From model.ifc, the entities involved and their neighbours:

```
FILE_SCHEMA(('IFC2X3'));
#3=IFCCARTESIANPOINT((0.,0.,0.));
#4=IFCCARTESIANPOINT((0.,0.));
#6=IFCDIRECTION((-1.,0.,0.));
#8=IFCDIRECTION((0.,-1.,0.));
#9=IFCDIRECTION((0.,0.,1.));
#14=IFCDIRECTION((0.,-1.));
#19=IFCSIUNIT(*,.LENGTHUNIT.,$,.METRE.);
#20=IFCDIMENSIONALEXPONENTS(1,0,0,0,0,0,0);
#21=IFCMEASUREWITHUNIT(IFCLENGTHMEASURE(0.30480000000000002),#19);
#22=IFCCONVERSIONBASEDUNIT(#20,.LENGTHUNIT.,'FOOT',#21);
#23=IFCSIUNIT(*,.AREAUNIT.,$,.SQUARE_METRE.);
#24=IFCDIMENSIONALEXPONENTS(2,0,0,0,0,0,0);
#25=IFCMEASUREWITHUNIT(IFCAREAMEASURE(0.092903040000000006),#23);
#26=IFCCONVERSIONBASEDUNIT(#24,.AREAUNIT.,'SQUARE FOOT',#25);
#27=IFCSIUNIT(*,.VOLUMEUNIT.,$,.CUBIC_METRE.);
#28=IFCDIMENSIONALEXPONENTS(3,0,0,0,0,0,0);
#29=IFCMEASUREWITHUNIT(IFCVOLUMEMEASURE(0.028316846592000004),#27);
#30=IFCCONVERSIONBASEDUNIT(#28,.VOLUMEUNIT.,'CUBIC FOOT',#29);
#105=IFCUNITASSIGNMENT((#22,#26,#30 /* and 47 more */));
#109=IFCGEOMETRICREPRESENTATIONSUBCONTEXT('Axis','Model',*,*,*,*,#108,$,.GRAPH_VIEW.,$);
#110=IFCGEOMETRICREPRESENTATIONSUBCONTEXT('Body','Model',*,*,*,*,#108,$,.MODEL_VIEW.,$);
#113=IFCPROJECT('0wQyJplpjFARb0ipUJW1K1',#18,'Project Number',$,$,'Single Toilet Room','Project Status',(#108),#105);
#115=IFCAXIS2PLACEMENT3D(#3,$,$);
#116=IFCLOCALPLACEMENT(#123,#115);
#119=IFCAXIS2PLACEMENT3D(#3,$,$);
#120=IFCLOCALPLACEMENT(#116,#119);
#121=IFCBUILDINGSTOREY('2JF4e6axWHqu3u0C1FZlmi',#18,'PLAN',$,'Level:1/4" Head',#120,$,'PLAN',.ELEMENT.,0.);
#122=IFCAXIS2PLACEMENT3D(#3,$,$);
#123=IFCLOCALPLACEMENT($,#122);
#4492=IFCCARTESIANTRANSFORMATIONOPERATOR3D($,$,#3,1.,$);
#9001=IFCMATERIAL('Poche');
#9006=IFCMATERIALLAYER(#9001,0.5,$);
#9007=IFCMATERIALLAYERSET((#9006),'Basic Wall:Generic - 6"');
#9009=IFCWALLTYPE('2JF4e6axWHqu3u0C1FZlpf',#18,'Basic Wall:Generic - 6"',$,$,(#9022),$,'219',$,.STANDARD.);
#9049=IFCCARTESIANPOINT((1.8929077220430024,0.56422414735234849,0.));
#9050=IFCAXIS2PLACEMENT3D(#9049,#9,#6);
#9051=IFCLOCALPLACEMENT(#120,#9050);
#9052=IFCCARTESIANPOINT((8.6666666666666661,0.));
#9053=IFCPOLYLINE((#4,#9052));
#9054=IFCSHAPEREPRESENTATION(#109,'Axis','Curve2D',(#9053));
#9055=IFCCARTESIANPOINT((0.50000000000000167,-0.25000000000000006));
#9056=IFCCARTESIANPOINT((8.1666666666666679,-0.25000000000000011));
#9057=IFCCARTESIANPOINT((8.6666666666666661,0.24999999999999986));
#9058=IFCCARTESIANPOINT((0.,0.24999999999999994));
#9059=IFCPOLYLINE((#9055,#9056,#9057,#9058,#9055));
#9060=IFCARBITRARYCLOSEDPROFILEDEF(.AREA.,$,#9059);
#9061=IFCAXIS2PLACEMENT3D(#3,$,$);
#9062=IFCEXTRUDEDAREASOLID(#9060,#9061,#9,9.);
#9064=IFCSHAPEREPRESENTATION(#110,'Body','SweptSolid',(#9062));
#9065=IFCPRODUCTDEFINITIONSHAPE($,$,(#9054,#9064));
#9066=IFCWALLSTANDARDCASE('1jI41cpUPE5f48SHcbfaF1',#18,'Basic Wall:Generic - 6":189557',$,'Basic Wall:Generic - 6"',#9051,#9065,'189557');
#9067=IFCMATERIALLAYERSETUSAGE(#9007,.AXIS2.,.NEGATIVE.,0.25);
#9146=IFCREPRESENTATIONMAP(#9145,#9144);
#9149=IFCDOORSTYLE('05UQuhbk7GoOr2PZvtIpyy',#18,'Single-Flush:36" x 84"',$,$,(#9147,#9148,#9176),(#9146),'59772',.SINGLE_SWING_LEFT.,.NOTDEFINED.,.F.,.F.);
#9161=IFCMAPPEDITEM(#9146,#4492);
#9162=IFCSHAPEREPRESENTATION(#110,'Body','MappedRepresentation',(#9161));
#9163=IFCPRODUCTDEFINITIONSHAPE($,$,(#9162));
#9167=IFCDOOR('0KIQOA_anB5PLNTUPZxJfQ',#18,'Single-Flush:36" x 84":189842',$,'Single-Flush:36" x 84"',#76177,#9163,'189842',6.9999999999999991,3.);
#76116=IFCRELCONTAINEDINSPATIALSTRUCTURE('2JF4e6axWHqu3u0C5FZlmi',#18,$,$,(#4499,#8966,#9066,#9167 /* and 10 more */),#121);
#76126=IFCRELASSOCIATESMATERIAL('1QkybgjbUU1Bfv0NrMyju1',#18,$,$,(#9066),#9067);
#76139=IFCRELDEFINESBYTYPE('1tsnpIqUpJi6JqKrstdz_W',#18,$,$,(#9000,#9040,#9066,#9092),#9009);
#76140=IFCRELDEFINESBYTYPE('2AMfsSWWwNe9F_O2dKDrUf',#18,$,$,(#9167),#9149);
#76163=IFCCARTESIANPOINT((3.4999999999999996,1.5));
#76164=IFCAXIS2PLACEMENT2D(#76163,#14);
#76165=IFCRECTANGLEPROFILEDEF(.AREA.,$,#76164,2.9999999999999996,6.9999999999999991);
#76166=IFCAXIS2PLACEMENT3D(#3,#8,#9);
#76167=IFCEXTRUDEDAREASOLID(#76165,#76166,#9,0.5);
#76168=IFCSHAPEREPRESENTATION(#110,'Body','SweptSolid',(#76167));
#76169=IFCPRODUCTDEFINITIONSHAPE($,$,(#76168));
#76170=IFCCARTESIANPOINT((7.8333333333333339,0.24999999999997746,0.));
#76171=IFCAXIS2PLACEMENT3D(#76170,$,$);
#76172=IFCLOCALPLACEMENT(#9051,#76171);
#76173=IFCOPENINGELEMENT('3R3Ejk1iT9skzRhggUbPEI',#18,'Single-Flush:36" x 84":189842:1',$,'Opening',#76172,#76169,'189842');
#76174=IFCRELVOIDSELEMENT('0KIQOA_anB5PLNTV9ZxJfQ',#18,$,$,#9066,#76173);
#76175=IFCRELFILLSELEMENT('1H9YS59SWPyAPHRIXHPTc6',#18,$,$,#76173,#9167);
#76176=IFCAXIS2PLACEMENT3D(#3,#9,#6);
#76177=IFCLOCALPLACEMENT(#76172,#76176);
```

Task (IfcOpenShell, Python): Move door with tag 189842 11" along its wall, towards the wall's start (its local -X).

```python
import ifcopenshell
import ifcopenshell.api.geometry
import ifcopenshell.util.placement
import ifcopenshell.util.unit

model = ifcopenshell.open("model.ifc")
unit_scale = ifcopenshell.util.unit.calculate_unit_scale(model)

door = model.by_id(9167)
opening = door.FillsVoids[0].RelatingOpeningElement
wall = opening.VoidsElements[0].RelatingBuildingElement

wall_matrix = ifcopenshell.util.placement.get_local_placement(wall.ObjectPlacement)
shift = wall_matrix[:3, 0] * -11 * 0.0254 / unit_scale
before = ifcopenshell.util.placement.get_local_placement(door.ObjectPlacement)[:3, 3].copy()

# The door is placed relative to its opening, so it follows when the opening moves.
matrix = ifcopenshell.util.placement.get_local_placement(opening.ObjectPlacement)
matrix[:3, 3] += shift
ifcopenshell.api.geometry.edit_object_placement(
    model, product=opening, matrix=matrix, is_si=False, should_transform_children=True
)

after = ifcopenshell.util.placement.get_local_placement(door.ObjectPlacement)[:3, 3]
print("door moved by", (after - before).round(3) + 0.0)

model.write("model-out.ifc")
```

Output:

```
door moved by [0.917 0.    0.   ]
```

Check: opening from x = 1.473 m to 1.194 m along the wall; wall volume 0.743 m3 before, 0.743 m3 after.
